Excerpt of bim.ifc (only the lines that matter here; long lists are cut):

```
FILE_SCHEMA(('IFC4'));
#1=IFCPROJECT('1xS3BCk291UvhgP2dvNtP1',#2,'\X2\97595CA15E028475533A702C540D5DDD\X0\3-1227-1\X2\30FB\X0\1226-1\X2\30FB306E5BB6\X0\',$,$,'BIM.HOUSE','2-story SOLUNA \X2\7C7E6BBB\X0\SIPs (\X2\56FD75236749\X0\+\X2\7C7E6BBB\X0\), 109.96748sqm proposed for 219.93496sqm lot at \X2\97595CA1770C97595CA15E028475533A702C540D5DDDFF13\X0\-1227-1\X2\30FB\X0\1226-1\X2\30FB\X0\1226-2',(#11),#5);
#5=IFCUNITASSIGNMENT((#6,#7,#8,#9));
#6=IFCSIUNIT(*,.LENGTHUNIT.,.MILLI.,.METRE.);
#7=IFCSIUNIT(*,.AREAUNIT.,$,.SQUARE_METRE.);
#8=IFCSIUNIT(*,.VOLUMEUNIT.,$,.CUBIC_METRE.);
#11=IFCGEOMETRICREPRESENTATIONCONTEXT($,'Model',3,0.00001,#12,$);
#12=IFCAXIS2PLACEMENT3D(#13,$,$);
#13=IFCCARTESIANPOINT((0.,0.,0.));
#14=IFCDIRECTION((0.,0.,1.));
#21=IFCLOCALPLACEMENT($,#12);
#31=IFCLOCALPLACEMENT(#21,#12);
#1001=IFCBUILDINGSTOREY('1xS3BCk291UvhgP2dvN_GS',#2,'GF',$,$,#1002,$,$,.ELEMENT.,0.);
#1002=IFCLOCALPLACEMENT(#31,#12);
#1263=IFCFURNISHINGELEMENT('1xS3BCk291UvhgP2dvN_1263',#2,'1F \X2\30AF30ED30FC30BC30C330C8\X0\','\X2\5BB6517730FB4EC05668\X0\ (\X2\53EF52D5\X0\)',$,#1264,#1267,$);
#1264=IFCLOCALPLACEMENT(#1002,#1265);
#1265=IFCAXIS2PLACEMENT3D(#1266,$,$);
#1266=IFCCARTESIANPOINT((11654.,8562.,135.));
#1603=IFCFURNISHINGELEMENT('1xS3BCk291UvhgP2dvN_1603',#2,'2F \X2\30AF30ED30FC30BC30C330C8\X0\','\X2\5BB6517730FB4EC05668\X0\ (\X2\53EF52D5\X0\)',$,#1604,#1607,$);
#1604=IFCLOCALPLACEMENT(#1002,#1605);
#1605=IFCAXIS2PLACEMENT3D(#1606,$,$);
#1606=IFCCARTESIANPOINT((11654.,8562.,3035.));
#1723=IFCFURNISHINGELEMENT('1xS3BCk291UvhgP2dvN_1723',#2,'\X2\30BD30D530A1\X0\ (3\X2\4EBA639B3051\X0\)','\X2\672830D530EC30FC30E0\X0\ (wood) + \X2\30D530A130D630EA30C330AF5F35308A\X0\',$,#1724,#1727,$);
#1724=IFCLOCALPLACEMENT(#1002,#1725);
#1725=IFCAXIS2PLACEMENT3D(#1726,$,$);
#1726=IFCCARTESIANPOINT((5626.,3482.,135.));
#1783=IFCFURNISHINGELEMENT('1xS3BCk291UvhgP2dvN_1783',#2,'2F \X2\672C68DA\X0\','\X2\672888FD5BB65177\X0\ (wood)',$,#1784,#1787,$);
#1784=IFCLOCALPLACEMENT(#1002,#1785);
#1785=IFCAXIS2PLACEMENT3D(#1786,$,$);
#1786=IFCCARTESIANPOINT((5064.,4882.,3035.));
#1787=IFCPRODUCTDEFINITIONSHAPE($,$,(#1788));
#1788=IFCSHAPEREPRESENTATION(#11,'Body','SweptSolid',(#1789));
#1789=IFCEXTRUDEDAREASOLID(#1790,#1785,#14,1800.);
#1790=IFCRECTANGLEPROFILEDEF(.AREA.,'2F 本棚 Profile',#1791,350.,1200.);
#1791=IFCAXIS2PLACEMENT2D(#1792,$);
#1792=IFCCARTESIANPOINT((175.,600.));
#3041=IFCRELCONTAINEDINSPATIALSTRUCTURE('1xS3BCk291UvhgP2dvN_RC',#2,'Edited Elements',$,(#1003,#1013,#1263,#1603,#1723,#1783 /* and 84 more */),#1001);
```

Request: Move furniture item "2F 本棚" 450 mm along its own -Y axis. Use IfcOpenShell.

```python
import ifcopenshell
import ifcopenshell.api.geometry
import ifcopenshell.util.placement
import ifcopenshell.util.unit

model = ifcopenshell.open("bim.ifc")
unit_scale = ifcopenshell.util.unit.calculate_unit_scale(model)

item = model.by_guid("1xS3BCk291UvhgP2dvN_1783")
matrix = ifcopenshell.util.placement.get_local_placement(item.ObjectPlacement)
matrix[:3, 3] -= matrix[:3, 1] * 0.45 / unit_scale
ifcopenshell.api.geometry.edit_object_placement(model, product=item, matrix=matrix, is_si=False)

print(ifcopenshell.util.placement.get_local_placement(item.ObjectPlacement).round(3) + 0.0)

model.write("bim_edited.ifc")
```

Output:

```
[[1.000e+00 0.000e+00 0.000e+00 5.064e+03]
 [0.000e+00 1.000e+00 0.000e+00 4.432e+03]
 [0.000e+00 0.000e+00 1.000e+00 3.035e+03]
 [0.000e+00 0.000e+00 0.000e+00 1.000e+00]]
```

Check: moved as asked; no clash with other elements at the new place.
